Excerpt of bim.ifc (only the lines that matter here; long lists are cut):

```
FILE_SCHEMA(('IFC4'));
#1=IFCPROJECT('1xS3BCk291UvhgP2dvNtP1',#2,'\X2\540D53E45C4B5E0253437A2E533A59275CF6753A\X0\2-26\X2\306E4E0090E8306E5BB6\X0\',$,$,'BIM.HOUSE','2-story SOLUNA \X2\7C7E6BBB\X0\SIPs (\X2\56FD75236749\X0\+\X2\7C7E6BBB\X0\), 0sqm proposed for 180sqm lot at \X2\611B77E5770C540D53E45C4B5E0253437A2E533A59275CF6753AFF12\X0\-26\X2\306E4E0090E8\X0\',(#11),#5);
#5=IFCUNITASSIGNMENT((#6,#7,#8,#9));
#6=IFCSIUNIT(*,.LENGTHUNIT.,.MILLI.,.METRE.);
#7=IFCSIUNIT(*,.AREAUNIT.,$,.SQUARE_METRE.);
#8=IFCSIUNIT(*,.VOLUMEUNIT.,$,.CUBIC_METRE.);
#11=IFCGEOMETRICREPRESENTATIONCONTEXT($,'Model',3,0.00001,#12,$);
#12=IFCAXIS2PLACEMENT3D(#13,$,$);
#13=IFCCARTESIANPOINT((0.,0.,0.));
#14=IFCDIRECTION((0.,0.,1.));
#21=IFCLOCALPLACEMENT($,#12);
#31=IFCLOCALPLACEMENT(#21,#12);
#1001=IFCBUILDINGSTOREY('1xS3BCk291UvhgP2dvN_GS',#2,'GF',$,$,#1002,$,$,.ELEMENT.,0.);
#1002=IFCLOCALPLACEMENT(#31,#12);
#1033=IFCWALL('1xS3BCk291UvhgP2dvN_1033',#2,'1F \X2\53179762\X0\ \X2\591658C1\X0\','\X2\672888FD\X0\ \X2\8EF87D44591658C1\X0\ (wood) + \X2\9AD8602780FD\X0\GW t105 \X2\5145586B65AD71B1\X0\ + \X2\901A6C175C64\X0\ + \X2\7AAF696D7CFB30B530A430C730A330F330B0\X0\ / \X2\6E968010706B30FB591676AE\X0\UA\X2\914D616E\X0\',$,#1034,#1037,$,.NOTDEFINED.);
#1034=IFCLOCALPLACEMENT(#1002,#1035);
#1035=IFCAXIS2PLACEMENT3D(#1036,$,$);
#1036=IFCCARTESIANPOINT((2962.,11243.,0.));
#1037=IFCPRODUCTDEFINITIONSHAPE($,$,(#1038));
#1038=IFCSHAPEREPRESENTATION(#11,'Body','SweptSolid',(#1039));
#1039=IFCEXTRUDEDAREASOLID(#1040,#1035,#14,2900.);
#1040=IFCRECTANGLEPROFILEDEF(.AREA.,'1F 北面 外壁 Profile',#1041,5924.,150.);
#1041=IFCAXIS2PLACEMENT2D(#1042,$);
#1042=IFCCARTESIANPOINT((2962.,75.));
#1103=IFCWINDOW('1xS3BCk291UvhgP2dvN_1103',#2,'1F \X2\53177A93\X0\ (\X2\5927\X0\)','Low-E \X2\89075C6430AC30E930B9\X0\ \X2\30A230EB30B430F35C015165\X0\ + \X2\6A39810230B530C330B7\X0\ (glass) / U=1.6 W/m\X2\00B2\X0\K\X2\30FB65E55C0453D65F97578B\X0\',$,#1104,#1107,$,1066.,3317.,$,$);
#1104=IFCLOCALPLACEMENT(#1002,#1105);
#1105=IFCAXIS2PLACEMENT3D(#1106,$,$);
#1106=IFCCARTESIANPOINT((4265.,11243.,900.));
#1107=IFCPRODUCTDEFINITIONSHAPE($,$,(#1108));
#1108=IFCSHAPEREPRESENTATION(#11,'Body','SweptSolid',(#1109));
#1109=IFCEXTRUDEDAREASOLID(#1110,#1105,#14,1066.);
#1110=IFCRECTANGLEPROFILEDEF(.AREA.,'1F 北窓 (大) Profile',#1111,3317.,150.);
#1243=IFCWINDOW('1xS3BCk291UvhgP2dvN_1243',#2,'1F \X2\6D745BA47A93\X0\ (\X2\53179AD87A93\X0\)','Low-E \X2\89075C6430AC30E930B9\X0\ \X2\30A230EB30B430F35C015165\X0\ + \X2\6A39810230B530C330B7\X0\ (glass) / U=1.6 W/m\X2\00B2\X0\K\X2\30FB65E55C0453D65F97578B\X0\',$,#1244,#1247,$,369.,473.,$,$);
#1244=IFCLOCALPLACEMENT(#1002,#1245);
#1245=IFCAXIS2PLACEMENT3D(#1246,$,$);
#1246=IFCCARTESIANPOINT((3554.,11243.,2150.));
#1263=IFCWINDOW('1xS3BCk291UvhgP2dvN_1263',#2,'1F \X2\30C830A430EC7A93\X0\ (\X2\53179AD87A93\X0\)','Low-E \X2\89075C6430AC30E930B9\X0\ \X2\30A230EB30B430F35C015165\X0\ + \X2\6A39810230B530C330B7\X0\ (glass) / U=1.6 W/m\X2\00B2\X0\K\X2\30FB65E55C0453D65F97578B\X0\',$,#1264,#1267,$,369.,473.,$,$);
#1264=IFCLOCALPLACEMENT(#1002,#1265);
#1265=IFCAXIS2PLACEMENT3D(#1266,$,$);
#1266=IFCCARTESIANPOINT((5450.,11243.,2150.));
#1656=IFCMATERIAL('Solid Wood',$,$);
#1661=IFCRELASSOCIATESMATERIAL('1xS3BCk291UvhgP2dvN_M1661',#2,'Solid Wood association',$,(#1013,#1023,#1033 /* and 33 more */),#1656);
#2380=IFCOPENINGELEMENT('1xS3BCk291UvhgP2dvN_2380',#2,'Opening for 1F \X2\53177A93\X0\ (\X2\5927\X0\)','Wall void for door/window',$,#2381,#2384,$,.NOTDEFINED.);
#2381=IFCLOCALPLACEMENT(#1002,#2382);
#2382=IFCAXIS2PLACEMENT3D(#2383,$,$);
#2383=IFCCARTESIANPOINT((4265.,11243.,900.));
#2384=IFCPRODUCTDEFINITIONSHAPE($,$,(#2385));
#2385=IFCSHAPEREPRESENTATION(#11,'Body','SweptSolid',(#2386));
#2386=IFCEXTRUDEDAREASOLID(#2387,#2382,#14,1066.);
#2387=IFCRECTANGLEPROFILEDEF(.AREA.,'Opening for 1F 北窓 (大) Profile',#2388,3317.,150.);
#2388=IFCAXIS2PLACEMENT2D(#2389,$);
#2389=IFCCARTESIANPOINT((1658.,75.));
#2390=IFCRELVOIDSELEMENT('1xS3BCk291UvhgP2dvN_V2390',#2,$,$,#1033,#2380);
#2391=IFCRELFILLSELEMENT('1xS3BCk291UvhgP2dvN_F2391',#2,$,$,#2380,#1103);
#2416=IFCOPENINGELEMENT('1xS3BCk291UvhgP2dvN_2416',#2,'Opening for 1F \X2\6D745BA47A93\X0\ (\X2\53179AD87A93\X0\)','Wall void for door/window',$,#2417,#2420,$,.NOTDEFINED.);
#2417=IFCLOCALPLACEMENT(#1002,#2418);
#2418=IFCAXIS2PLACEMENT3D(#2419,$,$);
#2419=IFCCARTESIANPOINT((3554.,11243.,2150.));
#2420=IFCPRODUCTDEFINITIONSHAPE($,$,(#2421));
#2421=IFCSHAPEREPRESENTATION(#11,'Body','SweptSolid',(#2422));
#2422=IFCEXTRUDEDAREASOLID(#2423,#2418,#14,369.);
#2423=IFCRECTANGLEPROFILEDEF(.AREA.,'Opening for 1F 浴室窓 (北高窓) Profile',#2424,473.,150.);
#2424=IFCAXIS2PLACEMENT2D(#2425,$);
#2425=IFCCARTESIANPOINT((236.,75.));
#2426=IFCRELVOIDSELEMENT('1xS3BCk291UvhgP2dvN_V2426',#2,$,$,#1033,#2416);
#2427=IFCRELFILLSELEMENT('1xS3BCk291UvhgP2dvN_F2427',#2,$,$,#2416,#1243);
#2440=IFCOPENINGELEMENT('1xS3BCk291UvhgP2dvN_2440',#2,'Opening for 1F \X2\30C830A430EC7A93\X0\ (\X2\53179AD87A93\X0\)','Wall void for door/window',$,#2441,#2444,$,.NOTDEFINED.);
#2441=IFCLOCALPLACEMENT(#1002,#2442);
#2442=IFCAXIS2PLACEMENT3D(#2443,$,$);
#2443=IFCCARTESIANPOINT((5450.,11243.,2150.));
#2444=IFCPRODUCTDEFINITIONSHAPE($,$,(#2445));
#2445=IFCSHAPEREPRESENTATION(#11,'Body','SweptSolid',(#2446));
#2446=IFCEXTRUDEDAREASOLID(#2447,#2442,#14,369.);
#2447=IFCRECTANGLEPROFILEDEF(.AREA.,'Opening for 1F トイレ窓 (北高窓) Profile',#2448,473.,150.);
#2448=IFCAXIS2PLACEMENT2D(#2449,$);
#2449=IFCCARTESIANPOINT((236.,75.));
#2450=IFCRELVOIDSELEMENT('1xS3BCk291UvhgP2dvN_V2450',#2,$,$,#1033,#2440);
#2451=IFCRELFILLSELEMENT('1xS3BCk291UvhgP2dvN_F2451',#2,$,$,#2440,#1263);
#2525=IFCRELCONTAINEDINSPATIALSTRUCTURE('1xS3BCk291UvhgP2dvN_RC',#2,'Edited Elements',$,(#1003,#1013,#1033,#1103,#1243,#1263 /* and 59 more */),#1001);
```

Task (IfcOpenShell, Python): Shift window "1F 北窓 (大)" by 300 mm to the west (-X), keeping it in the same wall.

```python
import ifcopenshell
import ifcopenshell.api.geometry
import ifcopenshell.util.placement
import ifcopenshell.util.unit

model = ifcopenshell.open("bim.ifc")
unit_scale = ifcopenshell.util.unit.calculate_unit_scale(model)

window = model.by_guid("1xS3BCk291UvhgP2dvN_1103")
opening = window.FillsVoids[0].RelatingOpeningElement
wall = opening.VoidsElements[0].RelatingBuildingElement

wall_matrix = ifcopenshell.util.placement.get_local_placement(wall.ObjectPlacement)
shift = wall_matrix[:3, 0] * -0.3 / unit_scale
before = ifcopenshell.util.placement.get_local_placement(window.ObjectPlacement)[:3, 3].copy()

# The window is not placed relative to its opening, so move both.
for product in (opening, window):
    matrix = ifcopenshell.util.placement.get_local_placement(product.ObjectPlacement)
    matrix[:3, 3] += shift
    ifcopenshell.api.geometry.edit_object_placement(model, product=product, matrix=matrix, is_si=False)

after = ifcopenshell.util.placement.get_local_placement(window.ObjectPlacement)[:3, 3]
print("window moved by", (after - before).round(3) + 0.0)

model.write("bim_v2.ifc")
```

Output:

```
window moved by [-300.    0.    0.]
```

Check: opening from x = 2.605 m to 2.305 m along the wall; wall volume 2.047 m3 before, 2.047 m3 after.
